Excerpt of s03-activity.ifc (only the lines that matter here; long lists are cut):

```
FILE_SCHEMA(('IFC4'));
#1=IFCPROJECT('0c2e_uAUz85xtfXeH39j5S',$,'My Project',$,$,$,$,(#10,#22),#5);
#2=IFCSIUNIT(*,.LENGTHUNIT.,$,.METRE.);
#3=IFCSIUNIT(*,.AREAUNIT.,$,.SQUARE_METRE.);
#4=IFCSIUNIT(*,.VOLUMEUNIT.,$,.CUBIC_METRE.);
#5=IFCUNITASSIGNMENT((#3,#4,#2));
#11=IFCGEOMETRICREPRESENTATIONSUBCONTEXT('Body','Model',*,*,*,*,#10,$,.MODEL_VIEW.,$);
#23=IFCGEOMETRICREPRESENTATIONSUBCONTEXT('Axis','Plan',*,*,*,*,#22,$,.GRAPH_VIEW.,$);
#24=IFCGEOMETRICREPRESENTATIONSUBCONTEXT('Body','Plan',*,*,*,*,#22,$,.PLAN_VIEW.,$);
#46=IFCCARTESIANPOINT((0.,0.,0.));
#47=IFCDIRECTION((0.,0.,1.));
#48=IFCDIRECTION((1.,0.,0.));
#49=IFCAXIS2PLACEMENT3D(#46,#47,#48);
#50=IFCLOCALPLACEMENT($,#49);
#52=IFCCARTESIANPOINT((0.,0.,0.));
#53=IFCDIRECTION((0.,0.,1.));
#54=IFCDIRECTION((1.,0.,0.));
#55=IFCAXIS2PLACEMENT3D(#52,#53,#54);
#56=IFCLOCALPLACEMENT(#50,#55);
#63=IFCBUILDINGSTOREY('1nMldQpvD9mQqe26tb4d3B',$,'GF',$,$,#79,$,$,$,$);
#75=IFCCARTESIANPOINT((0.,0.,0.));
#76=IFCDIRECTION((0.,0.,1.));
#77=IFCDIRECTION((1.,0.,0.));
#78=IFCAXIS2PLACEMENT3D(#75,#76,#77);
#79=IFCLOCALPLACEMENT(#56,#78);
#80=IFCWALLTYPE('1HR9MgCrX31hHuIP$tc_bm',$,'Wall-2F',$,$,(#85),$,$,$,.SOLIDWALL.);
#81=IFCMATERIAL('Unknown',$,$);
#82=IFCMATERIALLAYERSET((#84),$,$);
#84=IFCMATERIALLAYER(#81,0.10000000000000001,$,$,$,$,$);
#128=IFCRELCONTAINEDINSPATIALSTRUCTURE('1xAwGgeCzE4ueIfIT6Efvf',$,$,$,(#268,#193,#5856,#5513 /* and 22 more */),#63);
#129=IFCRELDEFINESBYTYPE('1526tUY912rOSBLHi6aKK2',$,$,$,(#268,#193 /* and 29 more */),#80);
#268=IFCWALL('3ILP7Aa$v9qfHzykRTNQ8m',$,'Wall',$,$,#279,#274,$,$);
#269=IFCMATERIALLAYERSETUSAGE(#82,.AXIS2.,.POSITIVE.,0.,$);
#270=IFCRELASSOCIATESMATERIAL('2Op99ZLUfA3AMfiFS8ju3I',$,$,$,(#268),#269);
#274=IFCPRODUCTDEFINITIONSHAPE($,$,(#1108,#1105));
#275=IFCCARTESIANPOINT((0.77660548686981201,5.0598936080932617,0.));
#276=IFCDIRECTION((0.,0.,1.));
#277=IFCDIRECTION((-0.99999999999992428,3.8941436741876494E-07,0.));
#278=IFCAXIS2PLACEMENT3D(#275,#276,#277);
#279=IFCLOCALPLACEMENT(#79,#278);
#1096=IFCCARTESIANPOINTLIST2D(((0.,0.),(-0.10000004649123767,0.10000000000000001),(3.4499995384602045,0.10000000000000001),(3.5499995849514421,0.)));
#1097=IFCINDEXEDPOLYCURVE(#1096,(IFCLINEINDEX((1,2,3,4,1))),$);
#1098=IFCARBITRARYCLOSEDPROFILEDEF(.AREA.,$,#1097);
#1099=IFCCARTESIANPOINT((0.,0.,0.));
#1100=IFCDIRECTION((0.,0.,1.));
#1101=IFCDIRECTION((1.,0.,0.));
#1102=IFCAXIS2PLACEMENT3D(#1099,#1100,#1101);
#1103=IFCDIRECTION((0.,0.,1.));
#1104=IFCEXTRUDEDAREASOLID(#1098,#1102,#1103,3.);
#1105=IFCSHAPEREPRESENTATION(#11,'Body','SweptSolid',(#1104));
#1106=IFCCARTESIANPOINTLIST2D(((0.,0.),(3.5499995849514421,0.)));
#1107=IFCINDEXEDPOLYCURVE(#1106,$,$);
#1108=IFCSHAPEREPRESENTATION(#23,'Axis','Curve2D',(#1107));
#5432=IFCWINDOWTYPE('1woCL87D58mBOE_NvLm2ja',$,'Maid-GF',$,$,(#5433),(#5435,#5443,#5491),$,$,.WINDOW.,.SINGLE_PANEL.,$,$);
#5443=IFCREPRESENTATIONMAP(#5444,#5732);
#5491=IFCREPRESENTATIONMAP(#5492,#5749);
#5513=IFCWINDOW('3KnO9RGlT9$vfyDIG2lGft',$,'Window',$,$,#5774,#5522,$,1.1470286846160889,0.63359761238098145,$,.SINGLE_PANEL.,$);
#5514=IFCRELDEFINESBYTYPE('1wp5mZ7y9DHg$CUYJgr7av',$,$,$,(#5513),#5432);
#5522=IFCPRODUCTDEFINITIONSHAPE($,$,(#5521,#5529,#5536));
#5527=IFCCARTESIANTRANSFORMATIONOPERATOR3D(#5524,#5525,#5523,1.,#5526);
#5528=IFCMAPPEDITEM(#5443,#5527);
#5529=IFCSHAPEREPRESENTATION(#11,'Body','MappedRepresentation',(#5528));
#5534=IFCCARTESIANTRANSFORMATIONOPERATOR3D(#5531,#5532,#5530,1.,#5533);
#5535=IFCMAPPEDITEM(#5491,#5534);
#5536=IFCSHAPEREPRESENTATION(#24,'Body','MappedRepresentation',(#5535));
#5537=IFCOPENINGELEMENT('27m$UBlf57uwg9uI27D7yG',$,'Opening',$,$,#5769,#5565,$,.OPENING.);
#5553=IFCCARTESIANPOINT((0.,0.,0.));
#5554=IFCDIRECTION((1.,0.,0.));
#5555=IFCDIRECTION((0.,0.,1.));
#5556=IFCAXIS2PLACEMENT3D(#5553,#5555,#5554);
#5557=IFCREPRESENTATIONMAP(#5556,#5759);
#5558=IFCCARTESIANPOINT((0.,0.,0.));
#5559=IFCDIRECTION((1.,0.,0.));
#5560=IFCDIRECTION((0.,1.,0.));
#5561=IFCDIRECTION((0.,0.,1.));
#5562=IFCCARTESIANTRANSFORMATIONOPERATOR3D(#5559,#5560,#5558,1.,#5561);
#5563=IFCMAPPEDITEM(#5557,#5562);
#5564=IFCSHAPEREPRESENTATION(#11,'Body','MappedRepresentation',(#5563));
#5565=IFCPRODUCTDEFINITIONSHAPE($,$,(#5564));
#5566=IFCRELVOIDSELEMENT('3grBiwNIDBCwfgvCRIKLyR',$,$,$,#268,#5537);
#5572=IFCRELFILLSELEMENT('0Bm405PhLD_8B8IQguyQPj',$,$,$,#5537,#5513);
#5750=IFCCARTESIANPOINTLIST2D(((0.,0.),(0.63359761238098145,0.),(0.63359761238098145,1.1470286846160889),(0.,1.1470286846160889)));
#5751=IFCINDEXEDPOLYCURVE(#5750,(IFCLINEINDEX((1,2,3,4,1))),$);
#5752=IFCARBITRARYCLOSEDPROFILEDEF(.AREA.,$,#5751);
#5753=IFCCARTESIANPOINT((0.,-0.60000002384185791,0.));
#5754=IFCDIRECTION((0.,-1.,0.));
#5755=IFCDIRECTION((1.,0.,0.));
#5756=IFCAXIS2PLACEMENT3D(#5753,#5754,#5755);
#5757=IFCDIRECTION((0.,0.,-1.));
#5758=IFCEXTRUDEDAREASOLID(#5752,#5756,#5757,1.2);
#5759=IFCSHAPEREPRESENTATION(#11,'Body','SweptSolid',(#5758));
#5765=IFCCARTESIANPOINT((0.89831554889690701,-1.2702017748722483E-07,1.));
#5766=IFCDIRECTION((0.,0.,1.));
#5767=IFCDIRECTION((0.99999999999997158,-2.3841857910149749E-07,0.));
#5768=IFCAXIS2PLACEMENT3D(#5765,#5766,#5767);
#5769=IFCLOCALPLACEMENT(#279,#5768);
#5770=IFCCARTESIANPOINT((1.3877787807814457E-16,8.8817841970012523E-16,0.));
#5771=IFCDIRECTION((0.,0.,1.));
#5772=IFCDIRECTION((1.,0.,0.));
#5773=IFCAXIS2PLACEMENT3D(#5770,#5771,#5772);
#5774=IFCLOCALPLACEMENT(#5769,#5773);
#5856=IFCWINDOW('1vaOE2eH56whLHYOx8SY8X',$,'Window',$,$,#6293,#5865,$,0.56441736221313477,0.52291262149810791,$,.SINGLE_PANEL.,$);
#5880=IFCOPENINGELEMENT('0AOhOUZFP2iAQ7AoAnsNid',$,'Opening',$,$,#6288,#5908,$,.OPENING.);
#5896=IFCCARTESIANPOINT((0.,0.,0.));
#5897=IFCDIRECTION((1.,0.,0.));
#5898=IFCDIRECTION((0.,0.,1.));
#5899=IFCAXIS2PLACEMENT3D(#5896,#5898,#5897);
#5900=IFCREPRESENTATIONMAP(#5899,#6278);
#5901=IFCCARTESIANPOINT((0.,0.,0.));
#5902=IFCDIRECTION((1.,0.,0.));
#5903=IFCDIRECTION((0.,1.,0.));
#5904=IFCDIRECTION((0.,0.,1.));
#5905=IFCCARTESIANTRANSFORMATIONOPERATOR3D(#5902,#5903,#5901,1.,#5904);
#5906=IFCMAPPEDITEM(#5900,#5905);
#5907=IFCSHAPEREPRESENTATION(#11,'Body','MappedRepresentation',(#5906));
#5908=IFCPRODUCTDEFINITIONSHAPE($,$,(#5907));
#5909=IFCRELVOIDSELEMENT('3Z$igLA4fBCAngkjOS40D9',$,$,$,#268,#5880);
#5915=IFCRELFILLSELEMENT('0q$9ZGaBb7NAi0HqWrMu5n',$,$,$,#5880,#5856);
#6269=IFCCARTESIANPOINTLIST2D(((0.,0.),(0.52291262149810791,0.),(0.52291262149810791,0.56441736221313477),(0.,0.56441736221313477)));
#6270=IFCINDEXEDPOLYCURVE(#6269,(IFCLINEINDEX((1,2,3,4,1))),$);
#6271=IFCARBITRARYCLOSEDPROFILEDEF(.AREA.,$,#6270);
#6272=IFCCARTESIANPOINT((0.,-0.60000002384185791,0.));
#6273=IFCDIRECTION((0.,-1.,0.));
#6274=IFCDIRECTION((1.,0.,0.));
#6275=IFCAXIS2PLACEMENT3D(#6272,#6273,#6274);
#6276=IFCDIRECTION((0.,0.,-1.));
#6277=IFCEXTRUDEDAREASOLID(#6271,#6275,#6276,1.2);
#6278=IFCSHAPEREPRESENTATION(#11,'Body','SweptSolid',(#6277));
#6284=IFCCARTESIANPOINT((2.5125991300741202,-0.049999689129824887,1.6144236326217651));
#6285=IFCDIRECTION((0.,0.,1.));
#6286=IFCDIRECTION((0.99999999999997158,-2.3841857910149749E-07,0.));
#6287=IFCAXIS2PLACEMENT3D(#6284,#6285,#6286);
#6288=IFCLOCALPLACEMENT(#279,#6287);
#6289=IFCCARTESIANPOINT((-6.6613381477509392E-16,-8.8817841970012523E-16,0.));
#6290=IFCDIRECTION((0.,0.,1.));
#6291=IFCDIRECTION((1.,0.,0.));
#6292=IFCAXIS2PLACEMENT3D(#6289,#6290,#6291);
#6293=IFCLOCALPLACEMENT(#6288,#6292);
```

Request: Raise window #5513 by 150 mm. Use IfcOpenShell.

```python
import numpy as np
import ifcopenshell
import ifcopenshell.api.geometry
import ifcopenshell.util.placement
import ifcopenshell.util.unit

model = ifcopenshell.open("s03-activity.ifc")
unit_scale = ifcopenshell.util.unit.calculate_unit_scale(model)

window = model.by_id(5513)
opening = window.FillsVoids[0].RelatingOpeningElement
dz = 0.15 / unit_scale

shift = np.array([0.0, 0.0, dz])
# The window is placed relative to its opening, so it follows when the opening moves.
matrix = ifcopenshell.util.placement.get_local_placement(opening.ObjectPlacement)
matrix[:3, 3] += shift
ifcopenshell.api.geometry.edit_object_placement(
    model, product=opening, matrix=matrix, is_si=False, should_transform_children=True
)

print(f"moved by {dz * unit_scale:+.3f} m")

model.write("s03-activity-out.ifc")
```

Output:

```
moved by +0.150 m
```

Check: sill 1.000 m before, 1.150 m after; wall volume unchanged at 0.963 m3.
